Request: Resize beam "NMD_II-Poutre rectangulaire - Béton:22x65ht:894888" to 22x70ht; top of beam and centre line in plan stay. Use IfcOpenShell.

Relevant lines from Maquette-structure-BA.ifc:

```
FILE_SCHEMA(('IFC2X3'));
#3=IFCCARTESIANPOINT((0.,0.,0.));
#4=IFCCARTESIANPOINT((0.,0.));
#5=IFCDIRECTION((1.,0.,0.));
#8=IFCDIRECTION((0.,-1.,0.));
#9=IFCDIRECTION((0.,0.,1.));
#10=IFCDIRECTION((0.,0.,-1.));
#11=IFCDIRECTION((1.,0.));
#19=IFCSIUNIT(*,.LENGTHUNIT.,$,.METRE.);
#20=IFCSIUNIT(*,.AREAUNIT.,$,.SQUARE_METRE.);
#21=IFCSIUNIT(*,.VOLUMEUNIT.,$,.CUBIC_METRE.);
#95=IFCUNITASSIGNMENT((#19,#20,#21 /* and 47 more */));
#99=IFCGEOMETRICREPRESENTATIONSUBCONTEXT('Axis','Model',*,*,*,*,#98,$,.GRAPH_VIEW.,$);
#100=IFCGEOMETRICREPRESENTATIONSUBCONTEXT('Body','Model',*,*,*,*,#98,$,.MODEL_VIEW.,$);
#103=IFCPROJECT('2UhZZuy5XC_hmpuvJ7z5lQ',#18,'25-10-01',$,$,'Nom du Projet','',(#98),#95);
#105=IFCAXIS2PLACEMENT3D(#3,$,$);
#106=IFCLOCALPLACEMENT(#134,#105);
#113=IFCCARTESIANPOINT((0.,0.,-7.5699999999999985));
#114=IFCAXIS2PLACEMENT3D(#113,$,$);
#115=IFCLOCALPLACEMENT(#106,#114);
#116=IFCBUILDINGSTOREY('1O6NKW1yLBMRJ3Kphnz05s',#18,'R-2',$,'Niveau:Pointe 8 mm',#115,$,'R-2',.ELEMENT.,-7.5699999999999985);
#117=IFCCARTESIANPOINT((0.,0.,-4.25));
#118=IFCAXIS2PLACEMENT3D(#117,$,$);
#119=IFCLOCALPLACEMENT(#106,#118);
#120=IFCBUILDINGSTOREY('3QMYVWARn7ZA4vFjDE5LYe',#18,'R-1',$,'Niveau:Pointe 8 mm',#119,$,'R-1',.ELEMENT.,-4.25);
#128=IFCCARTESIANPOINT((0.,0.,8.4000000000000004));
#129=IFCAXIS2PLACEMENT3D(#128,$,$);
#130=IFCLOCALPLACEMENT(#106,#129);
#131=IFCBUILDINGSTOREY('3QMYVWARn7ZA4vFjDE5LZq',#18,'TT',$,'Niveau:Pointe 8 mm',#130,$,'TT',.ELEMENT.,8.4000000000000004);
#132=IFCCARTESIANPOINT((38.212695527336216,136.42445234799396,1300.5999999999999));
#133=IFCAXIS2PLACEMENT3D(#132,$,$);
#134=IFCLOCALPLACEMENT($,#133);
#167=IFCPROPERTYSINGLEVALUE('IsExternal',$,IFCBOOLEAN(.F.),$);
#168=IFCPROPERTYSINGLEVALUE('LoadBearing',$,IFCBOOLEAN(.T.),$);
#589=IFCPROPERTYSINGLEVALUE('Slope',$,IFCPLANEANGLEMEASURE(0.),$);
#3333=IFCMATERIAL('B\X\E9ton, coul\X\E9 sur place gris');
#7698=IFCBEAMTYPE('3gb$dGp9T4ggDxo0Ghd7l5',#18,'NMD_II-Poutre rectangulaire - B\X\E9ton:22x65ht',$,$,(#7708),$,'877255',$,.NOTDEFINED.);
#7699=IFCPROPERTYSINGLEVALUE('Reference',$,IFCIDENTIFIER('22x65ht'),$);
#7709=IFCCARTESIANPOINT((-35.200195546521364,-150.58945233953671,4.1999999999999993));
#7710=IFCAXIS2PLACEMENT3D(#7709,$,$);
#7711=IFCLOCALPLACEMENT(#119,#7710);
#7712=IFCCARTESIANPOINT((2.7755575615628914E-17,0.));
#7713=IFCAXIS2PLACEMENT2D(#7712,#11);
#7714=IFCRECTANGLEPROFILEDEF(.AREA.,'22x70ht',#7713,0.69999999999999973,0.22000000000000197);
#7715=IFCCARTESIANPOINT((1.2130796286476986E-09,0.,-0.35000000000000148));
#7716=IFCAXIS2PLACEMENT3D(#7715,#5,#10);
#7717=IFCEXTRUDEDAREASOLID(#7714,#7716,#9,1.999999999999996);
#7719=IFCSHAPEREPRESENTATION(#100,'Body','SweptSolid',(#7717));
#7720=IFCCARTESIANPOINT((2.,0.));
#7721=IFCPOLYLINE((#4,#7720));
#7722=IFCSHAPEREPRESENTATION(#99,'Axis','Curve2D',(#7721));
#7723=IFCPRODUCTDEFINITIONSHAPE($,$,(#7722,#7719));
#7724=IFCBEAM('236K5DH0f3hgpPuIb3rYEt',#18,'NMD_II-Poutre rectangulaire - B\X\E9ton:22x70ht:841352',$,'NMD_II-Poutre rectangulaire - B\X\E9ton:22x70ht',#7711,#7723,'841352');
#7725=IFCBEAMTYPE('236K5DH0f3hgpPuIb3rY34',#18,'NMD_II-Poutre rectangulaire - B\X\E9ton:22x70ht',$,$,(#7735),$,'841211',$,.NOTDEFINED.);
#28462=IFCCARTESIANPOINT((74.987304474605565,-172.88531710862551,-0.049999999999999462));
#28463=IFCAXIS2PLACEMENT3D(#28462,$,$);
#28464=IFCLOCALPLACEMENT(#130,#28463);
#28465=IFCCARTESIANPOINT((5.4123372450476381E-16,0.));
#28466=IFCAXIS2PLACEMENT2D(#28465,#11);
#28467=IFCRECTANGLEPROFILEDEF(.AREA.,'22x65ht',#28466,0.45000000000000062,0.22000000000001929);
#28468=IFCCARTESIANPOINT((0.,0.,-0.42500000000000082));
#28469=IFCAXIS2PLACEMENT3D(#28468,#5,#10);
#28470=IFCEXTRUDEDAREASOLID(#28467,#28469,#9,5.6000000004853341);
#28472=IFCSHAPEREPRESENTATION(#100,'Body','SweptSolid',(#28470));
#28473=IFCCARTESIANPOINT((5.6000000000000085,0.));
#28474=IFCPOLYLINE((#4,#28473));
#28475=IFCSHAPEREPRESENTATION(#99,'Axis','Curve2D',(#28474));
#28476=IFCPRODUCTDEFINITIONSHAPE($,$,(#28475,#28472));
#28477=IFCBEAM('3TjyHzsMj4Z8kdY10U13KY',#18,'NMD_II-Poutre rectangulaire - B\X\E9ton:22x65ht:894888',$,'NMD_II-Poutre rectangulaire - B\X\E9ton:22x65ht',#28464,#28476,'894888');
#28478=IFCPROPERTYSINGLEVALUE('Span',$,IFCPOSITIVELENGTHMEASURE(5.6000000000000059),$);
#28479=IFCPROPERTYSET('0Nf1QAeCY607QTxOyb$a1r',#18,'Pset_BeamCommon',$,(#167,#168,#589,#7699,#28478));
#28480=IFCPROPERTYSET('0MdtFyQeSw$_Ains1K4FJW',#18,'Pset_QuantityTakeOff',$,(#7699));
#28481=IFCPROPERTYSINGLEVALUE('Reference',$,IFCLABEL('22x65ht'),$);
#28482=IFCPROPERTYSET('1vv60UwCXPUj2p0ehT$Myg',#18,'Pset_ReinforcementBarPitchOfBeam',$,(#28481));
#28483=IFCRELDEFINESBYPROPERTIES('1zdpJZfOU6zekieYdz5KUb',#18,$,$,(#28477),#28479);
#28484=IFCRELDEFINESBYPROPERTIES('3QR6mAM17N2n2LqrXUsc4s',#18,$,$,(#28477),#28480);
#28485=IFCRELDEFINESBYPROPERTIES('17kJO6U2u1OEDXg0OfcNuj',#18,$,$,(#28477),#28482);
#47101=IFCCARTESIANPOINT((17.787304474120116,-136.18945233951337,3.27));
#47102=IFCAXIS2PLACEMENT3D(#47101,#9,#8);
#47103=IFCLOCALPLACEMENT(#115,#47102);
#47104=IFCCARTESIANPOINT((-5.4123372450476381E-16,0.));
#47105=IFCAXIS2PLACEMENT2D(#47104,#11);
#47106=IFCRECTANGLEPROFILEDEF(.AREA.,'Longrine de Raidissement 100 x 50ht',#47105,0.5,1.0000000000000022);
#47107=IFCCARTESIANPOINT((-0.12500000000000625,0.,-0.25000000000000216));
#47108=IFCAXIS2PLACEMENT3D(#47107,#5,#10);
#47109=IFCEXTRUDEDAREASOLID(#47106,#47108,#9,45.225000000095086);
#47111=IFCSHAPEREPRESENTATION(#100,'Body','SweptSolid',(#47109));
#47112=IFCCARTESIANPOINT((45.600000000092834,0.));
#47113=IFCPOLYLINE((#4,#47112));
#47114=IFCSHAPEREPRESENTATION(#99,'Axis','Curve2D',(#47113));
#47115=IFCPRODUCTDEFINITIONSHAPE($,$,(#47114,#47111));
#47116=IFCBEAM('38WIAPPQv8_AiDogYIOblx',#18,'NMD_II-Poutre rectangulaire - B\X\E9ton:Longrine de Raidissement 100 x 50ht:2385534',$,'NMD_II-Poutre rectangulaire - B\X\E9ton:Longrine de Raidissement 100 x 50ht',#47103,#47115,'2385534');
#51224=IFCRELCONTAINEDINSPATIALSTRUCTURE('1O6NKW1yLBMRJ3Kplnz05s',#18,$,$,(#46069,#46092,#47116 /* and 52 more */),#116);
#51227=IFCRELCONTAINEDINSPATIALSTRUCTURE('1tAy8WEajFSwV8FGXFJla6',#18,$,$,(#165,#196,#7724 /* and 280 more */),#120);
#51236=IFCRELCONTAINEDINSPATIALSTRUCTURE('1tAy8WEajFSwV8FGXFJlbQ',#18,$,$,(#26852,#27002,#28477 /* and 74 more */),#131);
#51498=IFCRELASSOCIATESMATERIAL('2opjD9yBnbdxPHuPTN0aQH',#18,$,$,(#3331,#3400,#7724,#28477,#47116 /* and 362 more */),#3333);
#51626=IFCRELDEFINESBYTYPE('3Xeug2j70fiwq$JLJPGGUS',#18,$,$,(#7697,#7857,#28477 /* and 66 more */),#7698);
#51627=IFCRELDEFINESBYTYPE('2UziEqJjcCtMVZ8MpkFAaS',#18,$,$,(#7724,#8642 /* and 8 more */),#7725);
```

```python
import ifcopenshell
import ifcopenshell.api.pset
import ifcopenshell.api.type
import ifcopenshell.util.element
import ifcopenshell.util.representation

model = ifcopenshell.open("Maquette-structure-BA.ifc")

member = model.by_guid("3TjyHzsMj4Z8kdY10U13KY")
source = next(p for p in model.by_type("IfcRectangleProfileDef") if p.ProfileName == "22x70ht")

body = ifcopenshell.util.representation.get_representation(member, "Model", "Body")
solid = body.Items[0]
old_profile = solid.SweptArea

# Copy the section's sizes but keep this member's own profile position.
profile = ifcopenshell.util.element.copy(model, source)
# Profiles are centred, so shift by half the change in depth to hold the top.
shift = (old_profile.XDim - profile.XDim) / 2
x, y = old_profile.Position.Location.Coordinates
up = (-1.0, 0.0)  # upwards, in the solid's own plane
location = model.createIfcCartesianPoint((x + up[0] * shift, y + up[1] * shift))
profile.Position = model.createIfcAxis2Placement2D(location, old_profile.Position.RefDirection)
solid.SweptArea = profile
if not model.get_total_inverses(old_profile):
    ifcopenshell.util.element.remove_deep2(model, old_profile)

new_type = model.by_guid("236K5DH0f3hgpPuIb3rY34")
ifcopenshell.api.type.assign_type(
    model, related_objects=[member], relating_type=new_type, should_map_representations=False
)
member.Name = member.Name.replace("22x65ht", "22x70ht")
member.ObjectType = "NMD_II-Poutre rectangulaire - Béton:22x70ht"
pset = model.by_id(ifcopenshell.util.element.get_pset(member, "Pset_BeamCommon", should_inherit=False)["id"])
ifcopenshell.api.pset.edit_pset(model, pset=pset, properties={"Reference": "22x70ht"})
pset = model.by_id(ifcopenshell.util.element.get_pset(member, "Pset_QuantityTakeOff", should_inherit=False)["id"])
ifcopenshell.api.pset.edit_pset(model, pset=pset, properties={"Reference": "22x70ht"})
pset = model.by_id(ifcopenshell.util.element.get_pset(member, "Pset_ReinforcementBarPitchOfBeam", should_inherit=False)["id"])
ifcopenshell.api.pset.edit_pset(model, pset=pset, properties={"Reference": "22x70ht"})

print(solid.SweptArea)

model.write("Maquette-structure-BA_edited.ifc")
```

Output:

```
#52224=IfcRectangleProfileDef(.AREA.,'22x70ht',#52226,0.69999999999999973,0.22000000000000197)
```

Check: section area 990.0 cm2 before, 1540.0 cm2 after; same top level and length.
